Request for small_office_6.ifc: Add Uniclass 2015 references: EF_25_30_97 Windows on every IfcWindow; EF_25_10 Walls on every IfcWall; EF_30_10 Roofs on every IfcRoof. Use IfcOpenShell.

First a look at what the model holds.

```python
import ifcopenshell

model = ifcopenshell.open("small_office_6.ifc")
print(model.schema)
print("classifications:", [c.Name for c in model.by_type("IfcClassification")])
for ifc_class in ("IfcDoor", "IfcRoof", "IfcStair", "IfcWall", "IfcWindow"):
    print(ifc_class, len(model.by_type(ifc_class)))
```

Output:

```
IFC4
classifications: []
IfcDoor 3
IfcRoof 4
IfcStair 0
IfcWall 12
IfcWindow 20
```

```python
import ifcopenshell
import ifcopenshell.api.classification

model = ifcopenshell.open("small_office_6.ifc")

system = ifcopenshell.api.classification.add_classification(model, classification="Uniclass 2015")

codes = {
    "IfcWindow": ("EF_25_30_97", "Windows"),
    "IfcWall": ("EF_25_10", "Walls"),
    "IfcRoof": ("EF_30_10", "Roofs"),
}
for ifc_class, (code, name) in codes.items():
    products = model.by_type(ifc_class)
    ifcopenshell.api.classification.add_reference(
        model, products=products, classification=system, identification=code, name=name
    )
    print(code, len(products))

model.write("small_office_6_rev.ifc")
```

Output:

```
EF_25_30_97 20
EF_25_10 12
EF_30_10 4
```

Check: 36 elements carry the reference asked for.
